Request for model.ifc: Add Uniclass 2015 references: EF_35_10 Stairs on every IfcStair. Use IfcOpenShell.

First a look at what the model holds.

```python
import ifcopenshell

model = ifcopenshell.open("model.ifc")
print(model.schema)
print("classifications:", [c.Name for c in model.by_type("IfcClassification")])
for ifc_class in ("IfcDoor", "IfcRoof", "IfcStair", "IfcWall", "IfcWindow"):
    print(ifc_class, len(model.by_type(ifc_class)))
```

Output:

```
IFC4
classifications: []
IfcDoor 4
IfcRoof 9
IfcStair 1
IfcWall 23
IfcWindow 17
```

```python
import ifcopenshell
import ifcopenshell.api.classification

model = ifcopenshell.open("model.ifc")

system = ifcopenshell.api.classification.add_classification(model, classification="Uniclass 2015")

codes = {
    "IfcStair": ("EF_35_10", "Stairs"),
}
for ifc_class, (code, name) in codes.items():
    products = model.by_type(ifc_class)
    ifcopenshell.api.classification.add_reference(
        model, products=products, classification=system, identification=code, name=name
    )
    print(code, len(products))

model.write("model-out.ifc")
```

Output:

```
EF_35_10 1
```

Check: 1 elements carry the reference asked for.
